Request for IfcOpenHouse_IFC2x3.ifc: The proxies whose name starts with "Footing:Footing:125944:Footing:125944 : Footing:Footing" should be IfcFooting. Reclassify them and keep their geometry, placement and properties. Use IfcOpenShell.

First a look at what the model holds.

```python
import re

import ifcopenshell

model = ifcopenshell.open("IfcOpenHouse_IFC2x3.ifc")
print(model.schema)
seen = {}
for e in model.by_type("IfcBuildingElementProxy"):
    name = re.sub(r":\d+(:\d+)?$", "", e.Name or "")  # drop the element id that some exporters append
    seen[name] = seen.get(name, 0) + 1
for name, count in sorted(seen.items()):
    print(count, "x", name)
```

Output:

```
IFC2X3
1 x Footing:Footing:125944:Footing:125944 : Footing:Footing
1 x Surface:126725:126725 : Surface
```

```python
import ifcopenshell
import ifcopenshell.api.root

model = ifcopenshell.open("IfcOpenHouse_IFC2x3.ifc")

proxies = [e.id() for e in model.by_type("IfcBuildingElementProxy") if (e.Name or "").startswith("Footing:Footing:125944:Footing:125944 : Footing:Footing")]
for step_id in proxies:
    proxy = model.by_id(step_id)
    ifcopenshell.api.root.reassign_class(model, product=proxy, ifc_class="IfcFooting", predefined_type="NOTDEFINED")

print(sum(model.by_id(i).is_a("IfcFooting") for i in proxies), "reclassified")

model.write("IfcOpenHouse_IFC2x3_edited.ifc")
```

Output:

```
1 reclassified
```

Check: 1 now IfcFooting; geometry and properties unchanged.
